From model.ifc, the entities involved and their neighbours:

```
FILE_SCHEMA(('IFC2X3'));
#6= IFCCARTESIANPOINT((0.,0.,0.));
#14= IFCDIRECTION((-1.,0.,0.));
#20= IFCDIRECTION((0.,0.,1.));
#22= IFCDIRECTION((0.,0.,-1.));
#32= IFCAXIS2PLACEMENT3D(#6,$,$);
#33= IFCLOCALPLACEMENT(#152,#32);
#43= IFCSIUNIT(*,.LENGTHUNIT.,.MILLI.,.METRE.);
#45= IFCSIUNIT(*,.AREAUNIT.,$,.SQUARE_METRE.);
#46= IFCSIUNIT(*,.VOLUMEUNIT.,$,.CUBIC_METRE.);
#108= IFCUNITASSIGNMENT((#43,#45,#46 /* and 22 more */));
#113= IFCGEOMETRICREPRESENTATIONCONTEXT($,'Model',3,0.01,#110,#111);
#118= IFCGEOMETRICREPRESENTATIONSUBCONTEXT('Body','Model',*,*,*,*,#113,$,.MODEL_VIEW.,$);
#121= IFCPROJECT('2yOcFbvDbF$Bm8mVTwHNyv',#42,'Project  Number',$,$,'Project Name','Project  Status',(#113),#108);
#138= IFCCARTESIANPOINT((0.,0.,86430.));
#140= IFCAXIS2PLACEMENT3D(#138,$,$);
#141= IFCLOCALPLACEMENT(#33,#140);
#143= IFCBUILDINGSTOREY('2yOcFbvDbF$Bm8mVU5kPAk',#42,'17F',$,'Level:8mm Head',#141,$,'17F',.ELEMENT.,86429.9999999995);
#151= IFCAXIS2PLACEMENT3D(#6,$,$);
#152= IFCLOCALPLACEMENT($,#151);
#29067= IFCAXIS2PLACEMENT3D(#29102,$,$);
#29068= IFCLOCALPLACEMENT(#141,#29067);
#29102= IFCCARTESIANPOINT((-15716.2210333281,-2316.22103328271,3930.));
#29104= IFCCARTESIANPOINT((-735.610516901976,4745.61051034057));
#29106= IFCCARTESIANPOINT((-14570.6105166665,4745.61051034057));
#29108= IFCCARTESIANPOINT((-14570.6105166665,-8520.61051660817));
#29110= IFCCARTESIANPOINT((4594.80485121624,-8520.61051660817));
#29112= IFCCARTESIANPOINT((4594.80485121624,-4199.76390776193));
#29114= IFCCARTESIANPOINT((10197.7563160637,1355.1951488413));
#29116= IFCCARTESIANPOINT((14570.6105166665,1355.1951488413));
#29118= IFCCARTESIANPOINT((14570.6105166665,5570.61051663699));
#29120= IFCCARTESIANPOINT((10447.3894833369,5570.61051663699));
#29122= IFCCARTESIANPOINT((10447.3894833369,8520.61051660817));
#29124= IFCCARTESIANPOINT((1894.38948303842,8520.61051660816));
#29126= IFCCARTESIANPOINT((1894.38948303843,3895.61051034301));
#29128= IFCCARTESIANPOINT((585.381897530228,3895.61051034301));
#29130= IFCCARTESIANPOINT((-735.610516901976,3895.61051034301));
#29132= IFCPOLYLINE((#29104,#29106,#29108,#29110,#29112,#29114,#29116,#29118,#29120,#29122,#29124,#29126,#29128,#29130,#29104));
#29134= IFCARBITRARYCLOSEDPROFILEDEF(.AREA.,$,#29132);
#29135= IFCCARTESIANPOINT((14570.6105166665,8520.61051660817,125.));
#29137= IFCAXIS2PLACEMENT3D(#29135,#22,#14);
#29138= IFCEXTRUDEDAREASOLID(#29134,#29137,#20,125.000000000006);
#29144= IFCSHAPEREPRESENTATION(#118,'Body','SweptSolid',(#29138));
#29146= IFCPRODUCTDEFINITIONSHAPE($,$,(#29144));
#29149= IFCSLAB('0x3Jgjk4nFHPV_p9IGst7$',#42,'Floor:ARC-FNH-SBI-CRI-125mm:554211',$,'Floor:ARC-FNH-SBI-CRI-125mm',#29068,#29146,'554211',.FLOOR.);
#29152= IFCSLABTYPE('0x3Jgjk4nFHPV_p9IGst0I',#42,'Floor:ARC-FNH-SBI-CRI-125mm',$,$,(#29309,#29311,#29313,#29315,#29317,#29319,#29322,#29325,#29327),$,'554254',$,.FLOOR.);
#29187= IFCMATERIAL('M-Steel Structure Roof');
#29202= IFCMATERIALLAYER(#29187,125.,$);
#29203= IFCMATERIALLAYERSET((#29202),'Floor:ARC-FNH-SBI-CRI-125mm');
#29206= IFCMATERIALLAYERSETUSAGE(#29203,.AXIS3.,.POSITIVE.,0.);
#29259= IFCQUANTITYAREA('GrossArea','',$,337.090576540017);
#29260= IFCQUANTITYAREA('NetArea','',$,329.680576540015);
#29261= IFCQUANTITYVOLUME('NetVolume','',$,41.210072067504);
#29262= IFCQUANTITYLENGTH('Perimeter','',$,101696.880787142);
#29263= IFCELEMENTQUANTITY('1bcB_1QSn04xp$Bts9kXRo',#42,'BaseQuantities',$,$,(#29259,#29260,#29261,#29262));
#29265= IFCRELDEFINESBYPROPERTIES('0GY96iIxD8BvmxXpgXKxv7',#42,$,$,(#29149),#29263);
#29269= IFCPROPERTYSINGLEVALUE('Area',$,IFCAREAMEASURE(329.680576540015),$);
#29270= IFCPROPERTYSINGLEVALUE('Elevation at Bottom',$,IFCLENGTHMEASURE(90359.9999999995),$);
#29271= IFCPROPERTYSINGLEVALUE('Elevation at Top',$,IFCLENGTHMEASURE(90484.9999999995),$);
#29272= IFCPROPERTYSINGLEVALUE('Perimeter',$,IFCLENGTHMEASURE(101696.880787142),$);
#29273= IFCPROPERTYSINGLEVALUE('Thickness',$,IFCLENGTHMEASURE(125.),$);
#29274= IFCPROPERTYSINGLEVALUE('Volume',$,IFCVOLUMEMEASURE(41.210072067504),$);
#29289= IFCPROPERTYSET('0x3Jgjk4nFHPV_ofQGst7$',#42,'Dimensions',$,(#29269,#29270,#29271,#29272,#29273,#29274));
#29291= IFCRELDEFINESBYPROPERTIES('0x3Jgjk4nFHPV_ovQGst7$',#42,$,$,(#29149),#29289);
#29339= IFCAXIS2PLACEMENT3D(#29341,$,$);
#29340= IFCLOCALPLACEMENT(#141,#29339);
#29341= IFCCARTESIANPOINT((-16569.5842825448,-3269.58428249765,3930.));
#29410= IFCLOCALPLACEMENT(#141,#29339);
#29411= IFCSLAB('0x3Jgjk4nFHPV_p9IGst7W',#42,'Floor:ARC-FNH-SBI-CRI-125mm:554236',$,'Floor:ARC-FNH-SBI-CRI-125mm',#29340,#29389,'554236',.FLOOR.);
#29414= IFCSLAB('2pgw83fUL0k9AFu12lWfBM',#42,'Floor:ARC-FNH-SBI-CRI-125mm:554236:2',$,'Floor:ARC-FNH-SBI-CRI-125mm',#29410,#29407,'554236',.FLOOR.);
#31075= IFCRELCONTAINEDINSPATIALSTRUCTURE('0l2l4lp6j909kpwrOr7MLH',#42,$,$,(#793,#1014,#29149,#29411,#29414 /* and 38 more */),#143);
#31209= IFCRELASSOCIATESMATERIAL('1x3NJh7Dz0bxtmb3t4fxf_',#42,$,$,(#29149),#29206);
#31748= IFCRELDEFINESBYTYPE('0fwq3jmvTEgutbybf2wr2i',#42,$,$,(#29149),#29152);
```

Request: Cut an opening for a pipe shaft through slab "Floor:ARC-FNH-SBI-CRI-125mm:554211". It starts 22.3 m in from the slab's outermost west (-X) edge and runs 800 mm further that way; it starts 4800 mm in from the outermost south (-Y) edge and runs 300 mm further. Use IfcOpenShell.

```python
import numpy as np
import ifcopenshell
import ifcopenshell.api.feature
import ifcopenshell.api.geometry
import ifcopenshell.api.pset
import ifcopenshell.api.root
import ifcopenshell.geom
import ifcopenshell.util.element
import ifcopenshell.util.placement
import ifcopenshell.util.representation
import ifcopenshell.util.shape
import ifcopenshell.util.unit

model = ifcopenshell.open("model.ifc")
unit_scale = ifcopenshell.util.unit.calculate_unit_scale(model)
area_scale = ifcopenshell.util.unit.calculate_unit_scale(model, "AREAUNIT")
volume_scale = ifcopenshell.util.unit.calculate_unit_scale(model, "VOLUMEUNIT")
settings = ifcopenshell.geom.settings()


def volume(element):
    """Net volume in cubic metres, openings subtracted."""
    shape = ifcopenshell.geom.create_shape(settings, element)
    return ifcopenshell.util.shape.get_volume(shape.geometry)


slab = model.by_guid("0x3Jgjk4nFHPV_p9IGst7$")
before = volume(slab)

# Extent in the slab's own axes, in metres. The edges named are its -X and -Y sides.
slab_shape = ifcopenshell.geom.create_shape(settings, slab)
vertices = ifcopenshell.util.shape.get_vertices(slab_shape.geometry)
x_min, y_min, bottom = vertices.min(axis=0)
top = vertices[:, 2].max()

opening = ifcopenshell.api.root.create_entity(model, ifc_class="IfcOpeningElement", name="Pipe shaft opening")
context = ifcopenshell.util.representation.get_context(model, "Model", "Body", "MODEL_VIEW")
width, depth = 0.8, 0.3
outline = [(0.0, 0.0), (width, 0.0), (width, depth), (0.0, depth), (0.0, 0.0)]
# Overshoot both faces by 50 mm so the cut is clean.
shape = ifcopenshell.api.geometry.add_slab_representation(
    model, context=context, depth=top - bottom + 0.1, polyline=outline
)
ifcopenshell.api.geometry.assign_representation(model, product=opening, representation=shape)

matrix = ifcopenshell.util.placement.get_local_placement(slab.ObjectPlacement)
matrix[:, 3] = matrix @ np.append(np.array([x_min + 22.3, y_min + 4.8, bottom - 0.05]) / unit_scale, 1.0)
ifcopenshell.api.geometry.edit_object_placement(model, product=opening, matrix=matrix, is_si=False)
ifcopenshell.api.feature.add_feature(model, feature=opening, element=slab)

after = volume(slab)

# Update the slab's stored quantities.
qto = model.by_id(ifcopenshell.util.element.get_pset(slab, "BaseQuantities", should_inherit=False)["id"])
ifcopenshell.api.pset.edit_qto(model, qto=qto, properties={
    "NetArea": after / (top - bottom) / area_scale,
    "NetVolume": after / volume_scale,
})
pset = model.by_id(ifcopenshell.util.element.get_pset(slab, "Dimensions", should_inherit=False)["id"])
ifcopenshell.api.pset.edit_pset(model, pset=pset, properties={
    "Area": model.create_entity("IfcAreaMeasure", after / (top - bottom) / area_scale),
    "Volume": model.create_entity("IfcVolumeMeasure", after / volume_scale),
})

print(f"slab volume {before:.3f} -> {after:.3f} m3")

model.write("model-out.ifc")
```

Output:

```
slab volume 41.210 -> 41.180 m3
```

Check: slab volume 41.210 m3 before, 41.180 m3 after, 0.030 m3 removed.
